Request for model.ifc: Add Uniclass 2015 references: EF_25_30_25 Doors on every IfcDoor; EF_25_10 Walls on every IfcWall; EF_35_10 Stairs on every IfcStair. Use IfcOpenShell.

First a look at what the model holds.

```python
import ifcopenshell

model = ifcopenshell.open("model.ifc")
print(model.schema)
print("classifications:", [c.Name for c in model.by_type("IfcClassification")])
for ifc_class in ("IfcDoor", "IfcRoof", "IfcStair", "IfcWall", "IfcWindow"):
    print(ifc_class, len(model.by_type(ifc_class)))
```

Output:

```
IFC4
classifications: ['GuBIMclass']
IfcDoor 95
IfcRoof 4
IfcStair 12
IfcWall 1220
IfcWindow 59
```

```python
import ifcopenshell
import ifcopenshell.api.classification

model = ifcopenshell.open("model.ifc")

system = ifcopenshell.api.classification.add_classification(model, classification="Uniclass 2015")

codes = {
    "IfcDoor": ("EF_25_30_25", "Doors"),
    "IfcWall": ("EF_25_10", "Walls"),
    "IfcStair": ("EF_35_10", "Stairs"),
}
for ifc_class, (code, name) in codes.items():
    products = model.by_type(ifc_class)
    ifcopenshell.api.classification.add_reference(
        model, products=products, classification=system, identification=code, name=name
    )
    print(code, len(products))

model.write("model_rev.ifc")
```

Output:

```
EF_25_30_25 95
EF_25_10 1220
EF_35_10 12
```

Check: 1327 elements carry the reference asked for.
